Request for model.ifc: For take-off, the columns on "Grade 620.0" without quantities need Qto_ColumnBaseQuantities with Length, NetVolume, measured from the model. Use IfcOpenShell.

First a look at what the model holds.

```python
import ifcopenshell
import ifcopenshell.util.element
import ifcopenshell.util.unit

model = ifcopenshell.open("model.ifc")
print(model.schema)
for unit_type in ("LENGTHUNIT", "AREAUNIT", "VOLUMEUNIT"):
    print(unit_type, ifcopenshell.util.unit.calculate_unit_scale(model, unit_type))
storey = next(s for s in model.by_type("IfcBuildingStorey") if s.Name == "Grade 620.0")
columns = [e for e in ifcopenshell.util.element.get_decomposition(storey) if e.is_a("IfcColumn")]
for e in sorted(columns, key=lambda e: e.id()):
    print(e.id(), e.is_a(), e.Name, list(ifcopenshell.util.element.get_psets(e, qtos_only=True)), sep=" | ")
```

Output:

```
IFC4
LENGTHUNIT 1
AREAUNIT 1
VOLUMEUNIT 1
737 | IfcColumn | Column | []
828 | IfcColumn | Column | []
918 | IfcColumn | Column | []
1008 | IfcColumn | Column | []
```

```python
import ifcopenshell
import ifcopenshell.api.pset
import ifcopenshell.geom
import ifcopenshell.util.element
import ifcopenshell.util.shape
import ifcopenshell.util.unit

model = ifcopenshell.open("model.ifc")
unit_scale = ifcopenshell.util.unit.calculate_unit_scale(model)
volume_scale = ifcopenshell.util.unit.calculate_unit_scale(model, "VOLUMEUNIT")
settings = ifcopenshell.geom.settings()

storey = next(s for s in model.by_type("IfcBuildingStorey") if s.Name == "Grade 620.0")
columns = [e for e in ifcopenshell.util.element.get_decomposition(storey) if e.is_a("IfcColumn")]

for e in sorted(columns, key=lambda e: e.id()):
    if ifcopenshell.util.element.get_psets(e, qtos_only=True, should_inherit=False):
        continue
    # Geometry comes back in metres, in the element's own axes.
    shape = ifcopenshell.geom.create_shape(settings, e)
    values = {
        "Length": ifcopenshell.util.shape.get_z(shape.geometry) / unit_scale,
        "NetVolume": ifcopenshell.util.shape.get_volume(shape.geometry) / volume_scale,
    }
    qto = ifcopenshell.api.pset.add_qto(model, product=e, name="Qto_ColumnBaseQuantities")
    ifcopenshell.api.pset.edit_qto(model, qto=qto, properties=values)
    print(e.id(), {k: round(v, 3) for k, v in values.items()})

model.write("model_updated.ifc")
```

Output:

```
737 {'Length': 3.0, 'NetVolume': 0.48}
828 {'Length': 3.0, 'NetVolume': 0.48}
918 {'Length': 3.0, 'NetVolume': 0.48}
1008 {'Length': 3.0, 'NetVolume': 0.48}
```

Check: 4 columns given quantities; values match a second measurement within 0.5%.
